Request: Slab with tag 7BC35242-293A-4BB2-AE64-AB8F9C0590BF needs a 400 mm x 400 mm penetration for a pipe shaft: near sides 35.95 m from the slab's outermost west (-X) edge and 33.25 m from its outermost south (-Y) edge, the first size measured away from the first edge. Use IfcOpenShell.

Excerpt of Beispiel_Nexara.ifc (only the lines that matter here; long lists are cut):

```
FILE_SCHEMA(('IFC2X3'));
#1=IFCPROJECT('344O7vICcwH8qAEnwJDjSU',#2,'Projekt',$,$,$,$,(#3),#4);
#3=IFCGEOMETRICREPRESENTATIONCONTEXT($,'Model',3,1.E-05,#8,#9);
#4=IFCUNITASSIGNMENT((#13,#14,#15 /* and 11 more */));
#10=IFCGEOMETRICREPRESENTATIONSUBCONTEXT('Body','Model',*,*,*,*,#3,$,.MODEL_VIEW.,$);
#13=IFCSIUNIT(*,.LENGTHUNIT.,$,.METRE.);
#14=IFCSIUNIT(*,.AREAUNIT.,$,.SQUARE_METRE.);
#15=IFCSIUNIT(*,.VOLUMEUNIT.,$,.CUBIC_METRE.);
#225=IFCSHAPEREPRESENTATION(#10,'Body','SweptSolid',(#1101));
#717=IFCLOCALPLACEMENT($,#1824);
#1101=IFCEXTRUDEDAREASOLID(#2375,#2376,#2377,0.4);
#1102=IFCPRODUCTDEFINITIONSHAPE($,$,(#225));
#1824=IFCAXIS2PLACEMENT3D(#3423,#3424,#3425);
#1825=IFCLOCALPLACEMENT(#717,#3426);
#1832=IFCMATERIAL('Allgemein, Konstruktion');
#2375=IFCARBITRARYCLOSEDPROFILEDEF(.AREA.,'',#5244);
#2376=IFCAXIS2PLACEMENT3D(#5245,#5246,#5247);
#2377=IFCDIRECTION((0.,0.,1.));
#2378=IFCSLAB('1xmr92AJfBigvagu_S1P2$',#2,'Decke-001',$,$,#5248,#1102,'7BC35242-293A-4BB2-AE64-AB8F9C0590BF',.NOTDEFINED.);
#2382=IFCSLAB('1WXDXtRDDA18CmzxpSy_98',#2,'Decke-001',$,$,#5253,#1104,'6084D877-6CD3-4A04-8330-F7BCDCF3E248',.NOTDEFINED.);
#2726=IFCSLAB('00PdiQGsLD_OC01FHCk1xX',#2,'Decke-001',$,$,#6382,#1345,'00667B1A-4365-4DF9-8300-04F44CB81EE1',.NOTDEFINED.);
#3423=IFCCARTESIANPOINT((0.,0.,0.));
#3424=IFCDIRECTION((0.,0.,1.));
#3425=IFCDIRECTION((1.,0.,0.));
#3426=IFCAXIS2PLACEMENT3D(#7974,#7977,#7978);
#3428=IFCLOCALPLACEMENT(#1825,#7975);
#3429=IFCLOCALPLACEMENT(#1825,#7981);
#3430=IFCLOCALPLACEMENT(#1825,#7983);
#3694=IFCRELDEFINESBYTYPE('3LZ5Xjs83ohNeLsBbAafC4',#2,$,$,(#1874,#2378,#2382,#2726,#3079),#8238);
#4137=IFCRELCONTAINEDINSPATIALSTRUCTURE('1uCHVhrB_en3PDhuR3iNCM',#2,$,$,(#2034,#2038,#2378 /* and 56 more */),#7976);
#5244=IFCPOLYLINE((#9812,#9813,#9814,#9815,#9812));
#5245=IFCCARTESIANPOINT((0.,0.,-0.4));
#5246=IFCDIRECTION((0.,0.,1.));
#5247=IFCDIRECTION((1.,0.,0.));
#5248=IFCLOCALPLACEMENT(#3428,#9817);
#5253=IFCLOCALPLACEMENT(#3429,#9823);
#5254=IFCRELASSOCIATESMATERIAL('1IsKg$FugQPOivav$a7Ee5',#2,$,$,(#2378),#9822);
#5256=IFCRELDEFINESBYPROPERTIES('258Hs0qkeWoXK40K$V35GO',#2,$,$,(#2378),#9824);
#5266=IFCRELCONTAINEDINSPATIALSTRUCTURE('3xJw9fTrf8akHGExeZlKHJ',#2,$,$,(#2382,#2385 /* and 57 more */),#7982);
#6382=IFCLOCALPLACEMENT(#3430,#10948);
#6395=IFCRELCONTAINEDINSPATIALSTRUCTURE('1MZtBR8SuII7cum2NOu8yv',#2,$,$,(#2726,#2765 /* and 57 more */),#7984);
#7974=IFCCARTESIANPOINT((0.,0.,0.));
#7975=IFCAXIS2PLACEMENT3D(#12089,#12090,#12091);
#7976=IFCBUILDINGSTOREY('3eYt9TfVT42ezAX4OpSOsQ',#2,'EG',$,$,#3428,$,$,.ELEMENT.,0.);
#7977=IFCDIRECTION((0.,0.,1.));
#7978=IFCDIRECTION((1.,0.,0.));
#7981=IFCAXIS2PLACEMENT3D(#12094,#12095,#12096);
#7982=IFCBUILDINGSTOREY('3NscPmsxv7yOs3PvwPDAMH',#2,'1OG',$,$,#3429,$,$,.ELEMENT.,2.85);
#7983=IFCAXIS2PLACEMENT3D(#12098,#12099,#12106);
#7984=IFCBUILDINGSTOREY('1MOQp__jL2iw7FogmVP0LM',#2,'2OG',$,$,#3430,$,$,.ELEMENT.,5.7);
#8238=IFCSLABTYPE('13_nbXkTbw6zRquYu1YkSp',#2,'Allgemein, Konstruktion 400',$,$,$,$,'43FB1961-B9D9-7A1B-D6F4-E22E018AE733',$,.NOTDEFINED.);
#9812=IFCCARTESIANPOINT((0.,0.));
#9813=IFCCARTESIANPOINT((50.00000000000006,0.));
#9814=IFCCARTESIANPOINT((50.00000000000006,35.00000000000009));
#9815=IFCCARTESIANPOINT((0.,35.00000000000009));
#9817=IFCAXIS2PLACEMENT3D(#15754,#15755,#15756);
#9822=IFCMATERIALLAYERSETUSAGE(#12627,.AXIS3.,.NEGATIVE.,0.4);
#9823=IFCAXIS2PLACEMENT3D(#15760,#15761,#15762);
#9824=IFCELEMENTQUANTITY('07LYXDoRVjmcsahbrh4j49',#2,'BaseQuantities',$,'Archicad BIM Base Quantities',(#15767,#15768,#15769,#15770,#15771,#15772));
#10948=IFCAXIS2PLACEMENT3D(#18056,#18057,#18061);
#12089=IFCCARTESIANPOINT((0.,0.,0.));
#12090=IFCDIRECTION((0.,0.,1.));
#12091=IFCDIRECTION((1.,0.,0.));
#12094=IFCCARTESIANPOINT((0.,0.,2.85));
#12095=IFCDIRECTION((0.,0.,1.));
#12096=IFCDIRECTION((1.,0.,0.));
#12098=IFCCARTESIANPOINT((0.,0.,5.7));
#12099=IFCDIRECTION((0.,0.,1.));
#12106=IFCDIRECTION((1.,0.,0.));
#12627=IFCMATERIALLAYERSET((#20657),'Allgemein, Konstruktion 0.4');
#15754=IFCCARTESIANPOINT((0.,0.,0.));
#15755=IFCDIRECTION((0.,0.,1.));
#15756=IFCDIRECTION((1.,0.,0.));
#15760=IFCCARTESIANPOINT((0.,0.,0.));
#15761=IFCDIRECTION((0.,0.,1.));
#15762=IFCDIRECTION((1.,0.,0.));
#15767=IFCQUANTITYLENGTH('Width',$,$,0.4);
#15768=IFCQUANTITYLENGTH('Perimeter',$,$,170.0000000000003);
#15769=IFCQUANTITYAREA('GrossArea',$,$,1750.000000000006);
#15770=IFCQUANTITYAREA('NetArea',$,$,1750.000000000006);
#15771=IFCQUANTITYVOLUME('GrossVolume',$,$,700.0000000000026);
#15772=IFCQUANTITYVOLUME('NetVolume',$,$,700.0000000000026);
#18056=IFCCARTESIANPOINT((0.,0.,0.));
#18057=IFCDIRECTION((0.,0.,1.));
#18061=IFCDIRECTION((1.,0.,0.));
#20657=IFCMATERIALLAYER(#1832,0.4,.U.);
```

```python
import numpy as np
import ifcopenshell
import ifcopenshell.api.feature
import ifcopenshell.api.geometry
import ifcopenshell.api.pset
import ifcopenshell.api.root
import ifcopenshell.geom
import ifcopenshell.util.element
import ifcopenshell.util.placement
import ifcopenshell.util.representation
import ifcopenshell.util.shape
import ifcopenshell.util.unit

model = ifcopenshell.open("Beispiel_Nexara.ifc")
unit_scale = ifcopenshell.util.unit.calculate_unit_scale(model)
area_scale = ifcopenshell.util.unit.calculate_unit_scale(model, "AREAUNIT")
volume_scale = ifcopenshell.util.unit.calculate_unit_scale(model, "VOLUMEUNIT")
settings = ifcopenshell.geom.settings()


def volume(element):
    """Net volume in cubic metres, openings subtracted."""
    shape = ifcopenshell.geom.create_shape(settings, element)
    return ifcopenshell.util.shape.get_volume(shape.geometry)


slab = model.by_guid("1xmr92AJfBigvagu_S1P2$")
before = volume(slab)

# Extent in the slab's own axes, in metres. The edges named are its -X and -Y sides.
slab_shape = ifcopenshell.geom.create_shape(settings, slab)
vertices = ifcopenshell.util.shape.get_vertices(slab_shape.geometry)
x_min, y_min, bottom = vertices.min(axis=0)
top = vertices[:, 2].max()

opening = ifcopenshell.api.root.create_entity(model, ifc_class="IfcOpeningElement", name="Pipe shaft opening")
context = ifcopenshell.util.representation.get_context(model, "Model", "Body", "MODEL_VIEW")
width, depth = 0.4, 0.4
outline = [(0.0, 0.0), (width, 0.0), (width, depth), (0.0, depth), (0.0, 0.0)]
# Overshoot both faces by 50 mm so the cut is clean.
shape = ifcopenshell.api.geometry.add_slab_representation(
    model, context=context, depth=top - bottom + 0.1, polyline=outline
)
ifcopenshell.api.geometry.assign_representation(model, product=opening, representation=shape)

matrix = ifcopenshell.util.placement.get_local_placement(slab.ObjectPlacement)
matrix[:, 3] = matrix @ np.append(np.array([x_min + 35.95, y_min + 33.25, bottom - 0.05]) / unit_scale, 1.0)
ifcopenshell.api.geometry.edit_object_placement(model, product=opening, matrix=matrix, is_si=False)
ifcopenshell.api.feature.add_feature(model, feature=opening, element=slab)

after = volume(slab)

# Update the slab's stored quantities.
qto = model.by_id(ifcopenshell.util.element.get_pset(slab, "BaseQuantities", should_inherit=False)["id"])
ifcopenshell.api.pset.edit_qto(model, qto=qto, properties={
    "NetArea": after / (top - bottom) / area_scale,
    "NetVolume": after / volume_scale,
})

print(f"slab volume {before:.3f} -> {after:.3f} m3")

model.write("Beispiel_Nexara_updated.ifc")
```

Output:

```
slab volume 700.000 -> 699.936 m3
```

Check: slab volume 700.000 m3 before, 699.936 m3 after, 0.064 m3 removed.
